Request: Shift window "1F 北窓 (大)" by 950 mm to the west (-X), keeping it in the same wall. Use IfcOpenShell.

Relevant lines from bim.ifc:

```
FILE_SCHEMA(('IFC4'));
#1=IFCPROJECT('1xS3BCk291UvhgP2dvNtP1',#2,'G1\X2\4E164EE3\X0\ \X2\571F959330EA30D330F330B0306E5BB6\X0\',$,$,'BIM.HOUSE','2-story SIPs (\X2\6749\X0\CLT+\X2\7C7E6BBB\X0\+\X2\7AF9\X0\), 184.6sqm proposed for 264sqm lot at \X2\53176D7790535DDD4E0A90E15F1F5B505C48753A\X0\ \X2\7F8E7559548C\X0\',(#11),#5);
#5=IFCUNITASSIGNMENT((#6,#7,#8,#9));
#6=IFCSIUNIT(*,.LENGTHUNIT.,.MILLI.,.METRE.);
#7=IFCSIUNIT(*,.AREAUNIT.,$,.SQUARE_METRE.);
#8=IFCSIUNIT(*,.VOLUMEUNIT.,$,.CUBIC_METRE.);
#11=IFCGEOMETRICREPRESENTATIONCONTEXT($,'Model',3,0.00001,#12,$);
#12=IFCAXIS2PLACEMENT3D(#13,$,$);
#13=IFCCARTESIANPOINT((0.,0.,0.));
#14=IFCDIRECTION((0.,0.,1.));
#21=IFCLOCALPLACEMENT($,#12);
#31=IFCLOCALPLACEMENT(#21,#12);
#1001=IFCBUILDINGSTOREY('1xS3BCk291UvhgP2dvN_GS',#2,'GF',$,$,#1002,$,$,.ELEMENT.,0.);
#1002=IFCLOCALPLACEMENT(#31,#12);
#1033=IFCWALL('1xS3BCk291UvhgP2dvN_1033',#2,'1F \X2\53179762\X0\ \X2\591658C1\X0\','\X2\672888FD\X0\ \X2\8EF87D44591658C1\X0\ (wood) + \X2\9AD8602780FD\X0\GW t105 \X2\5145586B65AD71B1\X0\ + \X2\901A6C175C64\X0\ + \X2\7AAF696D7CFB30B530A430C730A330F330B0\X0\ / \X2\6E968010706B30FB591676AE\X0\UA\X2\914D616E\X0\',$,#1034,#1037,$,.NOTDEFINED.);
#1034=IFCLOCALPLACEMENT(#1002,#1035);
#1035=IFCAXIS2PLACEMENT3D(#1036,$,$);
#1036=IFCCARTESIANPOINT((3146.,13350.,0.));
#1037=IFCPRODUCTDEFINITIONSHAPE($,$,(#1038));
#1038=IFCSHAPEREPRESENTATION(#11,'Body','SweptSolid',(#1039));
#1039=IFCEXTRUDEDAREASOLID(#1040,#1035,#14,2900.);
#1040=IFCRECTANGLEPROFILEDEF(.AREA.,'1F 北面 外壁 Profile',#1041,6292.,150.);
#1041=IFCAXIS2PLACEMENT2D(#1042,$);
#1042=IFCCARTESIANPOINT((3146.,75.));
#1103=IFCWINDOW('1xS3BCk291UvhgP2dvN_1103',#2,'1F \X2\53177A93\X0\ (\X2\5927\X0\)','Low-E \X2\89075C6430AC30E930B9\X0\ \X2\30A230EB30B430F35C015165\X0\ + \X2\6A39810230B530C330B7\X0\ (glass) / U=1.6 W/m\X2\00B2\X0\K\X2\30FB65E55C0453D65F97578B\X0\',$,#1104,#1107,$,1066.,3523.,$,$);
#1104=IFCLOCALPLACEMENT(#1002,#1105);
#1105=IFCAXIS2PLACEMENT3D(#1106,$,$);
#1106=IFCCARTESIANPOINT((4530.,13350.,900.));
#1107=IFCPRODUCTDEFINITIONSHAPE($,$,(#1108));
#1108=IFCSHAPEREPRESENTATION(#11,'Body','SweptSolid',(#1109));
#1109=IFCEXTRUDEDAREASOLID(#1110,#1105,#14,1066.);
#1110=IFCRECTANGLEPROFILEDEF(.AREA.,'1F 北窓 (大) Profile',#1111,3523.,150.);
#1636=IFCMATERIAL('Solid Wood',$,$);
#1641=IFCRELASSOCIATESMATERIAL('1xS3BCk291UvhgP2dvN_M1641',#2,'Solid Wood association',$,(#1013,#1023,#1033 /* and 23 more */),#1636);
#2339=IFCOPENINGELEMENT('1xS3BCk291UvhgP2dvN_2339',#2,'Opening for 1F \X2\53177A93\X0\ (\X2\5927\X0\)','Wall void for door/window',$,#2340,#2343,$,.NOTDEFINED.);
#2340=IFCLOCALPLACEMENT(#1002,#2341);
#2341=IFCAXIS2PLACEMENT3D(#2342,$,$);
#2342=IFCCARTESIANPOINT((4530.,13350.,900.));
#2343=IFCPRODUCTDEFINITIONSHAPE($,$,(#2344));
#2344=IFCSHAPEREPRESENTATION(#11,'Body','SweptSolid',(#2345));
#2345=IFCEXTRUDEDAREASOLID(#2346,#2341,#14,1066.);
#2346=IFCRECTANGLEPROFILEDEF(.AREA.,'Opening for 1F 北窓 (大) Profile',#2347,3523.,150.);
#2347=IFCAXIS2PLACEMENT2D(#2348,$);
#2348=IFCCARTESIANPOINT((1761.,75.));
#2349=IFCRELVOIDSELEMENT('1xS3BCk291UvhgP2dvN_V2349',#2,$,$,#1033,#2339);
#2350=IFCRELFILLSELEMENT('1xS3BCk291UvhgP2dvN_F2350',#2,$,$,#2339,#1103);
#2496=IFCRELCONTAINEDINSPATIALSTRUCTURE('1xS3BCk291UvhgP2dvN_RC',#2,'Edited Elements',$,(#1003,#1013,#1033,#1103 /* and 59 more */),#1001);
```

```python
import ifcopenshell
import ifcopenshell.api.geometry
import ifcopenshell.util.placement

model = ifcopenshell.open("bim.ifc")

window = model.by_id(1103)
opening = window.FillsVoids[0].RelatingOpeningElement
wall = opening.VoidsElements[0].RelatingBuildingElement

wall_matrix = ifcopenshell.util.placement.get_local_placement(wall.ObjectPlacement)
shift = wall_matrix[:3, 0] * -950.0
before = ifcopenshell.util.placement.get_local_placement(window.ObjectPlacement)[:3, 3].copy()

# The window is not placed relative to its opening, so move both.
for product in (opening, window):
    matrix = ifcopenshell.util.placement.get_local_placement(product.ObjectPlacement)
    matrix[:3, 3] += shift
    ifcopenshell.api.geometry.edit_object_placement(model, product=product, matrix=matrix, is_si=False)

after = ifcopenshell.util.placement.get_local_placement(window.ObjectPlacement)[:3, 3]
print("window moved by", (after - before).round(3) + 0.0)

model.write("bim_rev.ifc")
```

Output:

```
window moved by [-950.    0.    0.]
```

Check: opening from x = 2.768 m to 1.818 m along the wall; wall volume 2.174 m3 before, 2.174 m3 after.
